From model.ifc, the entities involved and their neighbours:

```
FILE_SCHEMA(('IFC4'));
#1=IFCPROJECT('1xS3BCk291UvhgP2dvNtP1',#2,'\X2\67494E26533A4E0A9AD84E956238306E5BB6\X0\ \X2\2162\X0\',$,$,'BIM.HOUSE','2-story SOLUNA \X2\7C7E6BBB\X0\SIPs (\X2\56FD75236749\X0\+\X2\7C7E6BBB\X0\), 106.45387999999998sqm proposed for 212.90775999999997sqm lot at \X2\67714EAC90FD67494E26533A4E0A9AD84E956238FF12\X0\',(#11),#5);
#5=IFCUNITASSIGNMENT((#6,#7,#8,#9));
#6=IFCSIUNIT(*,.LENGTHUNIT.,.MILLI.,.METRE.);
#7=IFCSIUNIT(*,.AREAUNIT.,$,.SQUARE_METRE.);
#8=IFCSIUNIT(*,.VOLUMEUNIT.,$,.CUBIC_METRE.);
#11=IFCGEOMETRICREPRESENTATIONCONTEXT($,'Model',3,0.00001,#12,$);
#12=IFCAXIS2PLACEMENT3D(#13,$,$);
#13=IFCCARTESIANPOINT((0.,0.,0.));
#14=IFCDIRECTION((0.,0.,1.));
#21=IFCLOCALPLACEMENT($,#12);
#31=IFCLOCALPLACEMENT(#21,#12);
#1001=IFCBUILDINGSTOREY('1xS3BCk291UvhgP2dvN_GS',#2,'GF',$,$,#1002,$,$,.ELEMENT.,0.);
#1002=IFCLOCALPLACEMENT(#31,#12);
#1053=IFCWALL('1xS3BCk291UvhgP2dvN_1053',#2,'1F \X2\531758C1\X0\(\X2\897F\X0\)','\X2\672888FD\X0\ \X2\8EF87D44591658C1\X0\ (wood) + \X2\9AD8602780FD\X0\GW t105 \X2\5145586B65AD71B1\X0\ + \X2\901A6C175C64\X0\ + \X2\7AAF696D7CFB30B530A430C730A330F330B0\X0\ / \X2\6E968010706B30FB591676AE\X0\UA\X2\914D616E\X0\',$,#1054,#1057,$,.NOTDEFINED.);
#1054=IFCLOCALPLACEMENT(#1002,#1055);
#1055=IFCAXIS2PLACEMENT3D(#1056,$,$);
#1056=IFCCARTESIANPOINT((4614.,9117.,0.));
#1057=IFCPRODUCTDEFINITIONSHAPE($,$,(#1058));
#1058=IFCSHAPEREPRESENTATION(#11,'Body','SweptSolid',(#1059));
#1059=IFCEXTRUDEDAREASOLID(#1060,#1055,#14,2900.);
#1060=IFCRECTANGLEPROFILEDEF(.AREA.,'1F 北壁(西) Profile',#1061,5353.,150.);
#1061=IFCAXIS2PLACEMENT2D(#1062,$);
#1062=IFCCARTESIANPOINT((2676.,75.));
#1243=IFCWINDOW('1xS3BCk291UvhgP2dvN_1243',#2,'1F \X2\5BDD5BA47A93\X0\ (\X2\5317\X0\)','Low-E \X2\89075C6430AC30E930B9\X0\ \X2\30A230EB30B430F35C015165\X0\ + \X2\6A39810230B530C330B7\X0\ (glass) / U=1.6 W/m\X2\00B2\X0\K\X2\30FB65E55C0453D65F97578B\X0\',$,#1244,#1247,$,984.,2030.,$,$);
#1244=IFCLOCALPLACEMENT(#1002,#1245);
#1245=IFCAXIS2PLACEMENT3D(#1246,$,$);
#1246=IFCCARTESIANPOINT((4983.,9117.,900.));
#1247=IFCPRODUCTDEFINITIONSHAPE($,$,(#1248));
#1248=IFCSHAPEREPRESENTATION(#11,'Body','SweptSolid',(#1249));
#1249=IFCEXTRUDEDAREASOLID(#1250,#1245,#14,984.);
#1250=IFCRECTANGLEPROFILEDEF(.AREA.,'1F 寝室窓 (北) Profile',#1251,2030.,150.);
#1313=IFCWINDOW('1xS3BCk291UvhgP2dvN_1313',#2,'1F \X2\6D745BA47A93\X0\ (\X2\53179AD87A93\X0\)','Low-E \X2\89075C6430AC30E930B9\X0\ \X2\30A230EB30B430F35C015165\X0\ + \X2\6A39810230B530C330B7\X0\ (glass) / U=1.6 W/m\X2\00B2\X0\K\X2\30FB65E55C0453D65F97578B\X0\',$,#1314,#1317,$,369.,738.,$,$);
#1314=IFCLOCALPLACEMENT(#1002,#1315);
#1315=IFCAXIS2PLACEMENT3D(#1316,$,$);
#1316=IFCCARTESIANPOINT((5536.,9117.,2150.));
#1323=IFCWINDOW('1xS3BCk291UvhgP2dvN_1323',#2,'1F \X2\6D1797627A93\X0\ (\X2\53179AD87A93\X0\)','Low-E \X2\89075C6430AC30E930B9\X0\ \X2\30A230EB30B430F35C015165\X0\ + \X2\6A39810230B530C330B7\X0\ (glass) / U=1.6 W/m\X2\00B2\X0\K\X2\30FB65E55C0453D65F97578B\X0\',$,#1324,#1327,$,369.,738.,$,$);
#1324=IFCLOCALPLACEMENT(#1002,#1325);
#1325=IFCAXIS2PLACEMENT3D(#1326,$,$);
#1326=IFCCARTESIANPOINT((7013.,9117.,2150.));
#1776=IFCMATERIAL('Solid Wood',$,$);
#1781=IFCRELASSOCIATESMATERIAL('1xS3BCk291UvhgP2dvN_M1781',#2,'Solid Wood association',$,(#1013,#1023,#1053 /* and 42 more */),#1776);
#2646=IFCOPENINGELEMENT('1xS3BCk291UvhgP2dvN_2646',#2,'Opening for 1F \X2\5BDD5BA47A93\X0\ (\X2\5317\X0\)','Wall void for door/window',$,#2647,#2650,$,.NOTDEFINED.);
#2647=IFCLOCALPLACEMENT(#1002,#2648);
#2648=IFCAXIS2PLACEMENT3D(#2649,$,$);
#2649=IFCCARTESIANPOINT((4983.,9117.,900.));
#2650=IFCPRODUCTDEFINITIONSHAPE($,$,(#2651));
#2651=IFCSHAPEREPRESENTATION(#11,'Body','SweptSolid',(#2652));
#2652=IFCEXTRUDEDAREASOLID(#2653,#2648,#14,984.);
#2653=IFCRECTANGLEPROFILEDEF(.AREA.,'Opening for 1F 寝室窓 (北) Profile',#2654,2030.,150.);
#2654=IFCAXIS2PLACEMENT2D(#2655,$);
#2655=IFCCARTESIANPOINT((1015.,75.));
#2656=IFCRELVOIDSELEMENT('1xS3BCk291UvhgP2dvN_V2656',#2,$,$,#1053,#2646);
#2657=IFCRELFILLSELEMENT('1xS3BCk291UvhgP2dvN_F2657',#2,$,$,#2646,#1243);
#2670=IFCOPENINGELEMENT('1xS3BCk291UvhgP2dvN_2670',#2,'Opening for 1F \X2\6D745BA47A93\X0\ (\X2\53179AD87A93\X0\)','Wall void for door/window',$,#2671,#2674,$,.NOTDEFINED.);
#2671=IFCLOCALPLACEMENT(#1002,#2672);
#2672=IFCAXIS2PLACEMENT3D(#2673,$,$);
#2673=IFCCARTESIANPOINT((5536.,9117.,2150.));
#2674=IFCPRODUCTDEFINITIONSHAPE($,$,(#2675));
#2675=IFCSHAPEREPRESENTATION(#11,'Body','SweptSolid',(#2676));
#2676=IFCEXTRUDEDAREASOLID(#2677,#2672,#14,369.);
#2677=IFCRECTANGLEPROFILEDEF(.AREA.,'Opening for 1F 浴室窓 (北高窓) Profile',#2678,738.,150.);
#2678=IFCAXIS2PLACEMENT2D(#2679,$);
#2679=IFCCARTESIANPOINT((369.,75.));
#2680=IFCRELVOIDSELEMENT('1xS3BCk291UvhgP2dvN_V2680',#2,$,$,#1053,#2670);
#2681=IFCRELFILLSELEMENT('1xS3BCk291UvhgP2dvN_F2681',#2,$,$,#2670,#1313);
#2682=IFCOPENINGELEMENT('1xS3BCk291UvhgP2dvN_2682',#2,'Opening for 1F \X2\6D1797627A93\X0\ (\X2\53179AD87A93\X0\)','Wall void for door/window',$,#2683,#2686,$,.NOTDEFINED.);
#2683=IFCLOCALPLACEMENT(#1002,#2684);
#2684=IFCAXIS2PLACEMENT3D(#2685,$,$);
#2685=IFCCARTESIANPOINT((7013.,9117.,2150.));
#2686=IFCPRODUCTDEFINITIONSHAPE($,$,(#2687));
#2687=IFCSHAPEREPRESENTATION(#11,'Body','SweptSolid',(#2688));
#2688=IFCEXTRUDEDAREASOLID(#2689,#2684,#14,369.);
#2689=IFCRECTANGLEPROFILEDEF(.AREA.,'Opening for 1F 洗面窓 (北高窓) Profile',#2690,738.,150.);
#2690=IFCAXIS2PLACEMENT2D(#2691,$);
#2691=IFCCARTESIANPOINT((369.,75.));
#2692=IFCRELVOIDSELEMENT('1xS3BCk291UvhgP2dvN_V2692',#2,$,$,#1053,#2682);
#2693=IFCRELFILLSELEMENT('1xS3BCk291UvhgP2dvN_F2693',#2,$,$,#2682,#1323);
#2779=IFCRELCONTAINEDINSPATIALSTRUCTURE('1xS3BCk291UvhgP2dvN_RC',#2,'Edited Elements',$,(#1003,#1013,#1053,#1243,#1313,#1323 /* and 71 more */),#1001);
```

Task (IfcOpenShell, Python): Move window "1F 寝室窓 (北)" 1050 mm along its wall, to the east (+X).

```python
import ifcopenshell
import ifcopenshell.api.geometry
import ifcopenshell.util.placement
import ifcopenshell.util.unit

model = ifcopenshell.open("model.ifc")
unit_scale = ifcopenshell.util.unit.calculate_unit_scale(model)

window = model.by_guid("1xS3BCk291UvhgP2dvN_1243")
opening = window.FillsVoids[0].RelatingOpeningElement
wall = opening.VoidsElements[0].RelatingBuildingElement

wall_matrix = ifcopenshell.util.placement.get_local_placement(wall.ObjectPlacement)
shift = wall_matrix[:3, 0] * 1.05 / unit_scale
before = ifcopenshell.util.placement.get_local_placement(window.ObjectPlacement)[:3, 3].copy()

# The window is not placed relative to its opening, so move both.
for product in (opening, window):
    matrix = ifcopenshell.util.placement.get_local_placement(product.ObjectPlacement)
    matrix[:3, 3] += shift
    ifcopenshell.api.geometry.edit_object_placement(model, product=product, matrix=matrix, is_si=False)

after = ifcopenshell.util.placement.get_local_placement(window.ObjectPlacement)[:3, 3]
print("window moved by", (after - before).round(3) + 0.0)

model.write("model_v2.ifc")
```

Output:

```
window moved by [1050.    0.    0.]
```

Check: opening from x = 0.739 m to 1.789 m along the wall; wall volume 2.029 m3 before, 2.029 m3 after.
